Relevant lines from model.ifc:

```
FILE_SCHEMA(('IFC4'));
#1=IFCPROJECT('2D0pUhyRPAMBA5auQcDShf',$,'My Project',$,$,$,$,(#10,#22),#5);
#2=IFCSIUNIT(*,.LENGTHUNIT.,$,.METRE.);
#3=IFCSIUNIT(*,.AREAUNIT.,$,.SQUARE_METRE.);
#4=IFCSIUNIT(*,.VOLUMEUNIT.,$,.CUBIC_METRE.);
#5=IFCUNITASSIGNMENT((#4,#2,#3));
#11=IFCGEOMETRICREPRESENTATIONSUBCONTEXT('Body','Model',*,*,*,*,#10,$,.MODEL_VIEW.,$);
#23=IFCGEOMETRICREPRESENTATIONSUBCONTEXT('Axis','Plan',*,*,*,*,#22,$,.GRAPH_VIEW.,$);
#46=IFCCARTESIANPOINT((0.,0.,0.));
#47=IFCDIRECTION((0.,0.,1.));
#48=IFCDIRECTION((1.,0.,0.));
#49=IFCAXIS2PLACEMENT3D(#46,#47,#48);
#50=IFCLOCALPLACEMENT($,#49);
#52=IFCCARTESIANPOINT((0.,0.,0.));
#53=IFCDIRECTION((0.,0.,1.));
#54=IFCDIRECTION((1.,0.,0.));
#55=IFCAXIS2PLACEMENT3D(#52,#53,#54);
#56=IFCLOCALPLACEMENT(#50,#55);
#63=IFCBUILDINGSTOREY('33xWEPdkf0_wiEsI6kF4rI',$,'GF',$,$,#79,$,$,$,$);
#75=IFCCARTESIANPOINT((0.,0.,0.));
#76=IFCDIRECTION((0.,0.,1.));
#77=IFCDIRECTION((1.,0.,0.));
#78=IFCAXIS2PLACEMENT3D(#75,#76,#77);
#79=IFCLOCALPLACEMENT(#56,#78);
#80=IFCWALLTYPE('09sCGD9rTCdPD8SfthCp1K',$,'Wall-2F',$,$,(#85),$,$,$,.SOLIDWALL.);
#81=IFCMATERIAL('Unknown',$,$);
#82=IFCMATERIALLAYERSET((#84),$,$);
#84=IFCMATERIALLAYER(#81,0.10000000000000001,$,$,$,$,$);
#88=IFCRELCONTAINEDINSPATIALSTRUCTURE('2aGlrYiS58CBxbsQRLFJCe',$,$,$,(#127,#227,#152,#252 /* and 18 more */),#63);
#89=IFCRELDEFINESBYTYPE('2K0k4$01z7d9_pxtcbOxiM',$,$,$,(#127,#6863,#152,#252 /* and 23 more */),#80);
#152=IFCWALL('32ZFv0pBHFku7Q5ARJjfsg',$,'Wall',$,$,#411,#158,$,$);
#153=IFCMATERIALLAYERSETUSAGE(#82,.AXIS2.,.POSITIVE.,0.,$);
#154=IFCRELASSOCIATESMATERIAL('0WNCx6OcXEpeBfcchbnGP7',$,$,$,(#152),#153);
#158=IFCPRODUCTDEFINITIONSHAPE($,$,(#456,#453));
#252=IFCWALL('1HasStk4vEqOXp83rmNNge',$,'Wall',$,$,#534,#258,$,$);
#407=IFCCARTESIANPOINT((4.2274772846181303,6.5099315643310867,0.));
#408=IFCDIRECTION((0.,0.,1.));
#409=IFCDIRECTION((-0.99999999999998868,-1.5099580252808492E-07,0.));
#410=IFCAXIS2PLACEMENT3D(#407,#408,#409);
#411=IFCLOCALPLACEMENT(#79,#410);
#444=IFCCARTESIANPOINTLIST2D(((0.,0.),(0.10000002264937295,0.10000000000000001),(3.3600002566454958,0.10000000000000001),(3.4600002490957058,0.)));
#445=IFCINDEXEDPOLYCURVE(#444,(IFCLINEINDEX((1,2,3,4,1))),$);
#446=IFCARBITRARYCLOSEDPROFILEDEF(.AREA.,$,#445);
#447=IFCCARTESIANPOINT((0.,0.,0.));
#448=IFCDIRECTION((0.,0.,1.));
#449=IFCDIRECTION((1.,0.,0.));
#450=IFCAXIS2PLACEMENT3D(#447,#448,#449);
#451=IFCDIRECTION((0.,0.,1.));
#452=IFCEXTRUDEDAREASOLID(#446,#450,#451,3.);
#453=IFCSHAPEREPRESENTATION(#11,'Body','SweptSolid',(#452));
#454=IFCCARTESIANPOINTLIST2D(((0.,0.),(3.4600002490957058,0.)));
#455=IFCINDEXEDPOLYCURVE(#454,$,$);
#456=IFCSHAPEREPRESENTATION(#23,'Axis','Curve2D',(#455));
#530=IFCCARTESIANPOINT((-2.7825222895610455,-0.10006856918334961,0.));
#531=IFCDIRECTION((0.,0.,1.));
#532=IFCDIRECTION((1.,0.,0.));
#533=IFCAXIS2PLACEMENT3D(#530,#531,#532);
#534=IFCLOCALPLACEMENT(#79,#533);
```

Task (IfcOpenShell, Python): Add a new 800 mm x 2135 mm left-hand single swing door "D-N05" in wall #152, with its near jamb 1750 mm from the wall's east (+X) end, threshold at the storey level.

```python
import numpy as np
import ifcopenshell
import ifcopenshell.api.feature
import ifcopenshell.api.geometry
import ifcopenshell.api.root
import ifcopenshell.api.spatial
import ifcopenshell.geom
import ifcopenshell.util.element
import ifcopenshell.util.placement
import ifcopenshell.util.representation
import ifcopenshell.util.shape
import ifcopenshell.util.unit

model = ifcopenshell.open("model.ifc")
unit_scale = ifcopenshell.util.unit.calculate_unit_scale(model)
settings = ifcopenshell.geom.settings()


def volume(element):
    """Net volume in cubic metres, openings subtracted."""
    shape = ifcopenshell.geom.create_shape(settings, element)
    return ifcopenshell.util.shape.get_volume(shape.geometry)


wall = model.by_guid("32ZFv0pBHFku7Q5ARJjfsg")
storey = ifcopenshell.util.element.get_container(wall, ifc_class="IfcBuildingStorey")
context = ifcopenshell.util.representation.get_context(model, "Model", "Body", "MODEL_VIEW")
before = volume(wall)

width, height, from_end, sill = 0.8, 2.135, 1.75, 0.0  # metres

# The wall runs along its own X axis, and the end named is its -X end.
wall_shape = ifcopenshell.geom.create_shape(settings, wall)
x, y, z = ifcopenshell.util.shape.get_vertices(wall_shape.geometry).T
start = x.min() + from_end
face, thickness = float(y.min()), float(y.max() - y.min())
wall_matrix = ifcopenshell.util.placement.get_local_placement(wall.ObjectPlacement)
level = ifcopenshell.util.placement.get_local_placement(storey.ObjectPlacement)[2, 3]


def in_wall(x, y):
    """Placement at x, y metres in the wall's axes, at sill height."""
    matrix = wall_matrix.copy()
    matrix[:, 3] = wall_matrix @ np.array([x / unit_scale, y / unit_scale, 0.0, 1.0])
    matrix[2, 3] = level + sill / unit_scale
    return matrix


# Opening: a box that overshoots both wall faces by 50 mm.
opening = ifcopenshell.api.root.create_entity(model, ifc_class="IfcOpeningElement", predefined_type="OPENING")
box = ifcopenshell.api.geometry.add_wall_representation(
    model, context=context, length=width, height=height, thickness=thickness + 0.1
)
ifcopenshell.api.geometry.assign_representation(model, product=opening, representation=box)
ifcopenshell.api.geometry.edit_object_placement(model, product=opening, matrix=in_wall(start, face - 0.05), is_si=False)
ifcopenshell.api.feature.add_feature(model, feature=opening, element=wall)

door = ifcopenshell.api.root.create_entity(model, ifc_class="IfcDoor", name="D-N05", predefined_type="DOOR")
door.OverallWidth, door.OverallHeight = width / unit_scale, height / unit_scale
door.OperationType = "SINGLE_SWING_LEFT"
body = ifcopenshell.api.geometry.add_door_representation(
    model,
    context=context,
    overall_width=door.OverallWidth,
    overall_height=door.OverallHeight,
    operation_type="SINGLE_SWING_LEFT",
    lining_properties={"LiningDepth": thickness / unit_scale, "ThresholdDepth": thickness / unit_scale},
)
ifcopenshell.api.geometry.assign_representation(model, product=door, representation=body)
ifcopenshell.api.spatial.assign_container(model, products=[door], relating_structure=storey)
ifcopenshell.api.feature.add_filling(model, opening=opening, element=door)

# The lining spans the wall, so the door starts at the wall face.
ifcopenshell.api.geometry.edit_object_placement(model, product=door, matrix=in_wall(start, face), is_si=False)

after = volume(wall)

print(f"wall volume {before:.3f} -> {after:.3f} m3")

model.write("model-out.ifc")
```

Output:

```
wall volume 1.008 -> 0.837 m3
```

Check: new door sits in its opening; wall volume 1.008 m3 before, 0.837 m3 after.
